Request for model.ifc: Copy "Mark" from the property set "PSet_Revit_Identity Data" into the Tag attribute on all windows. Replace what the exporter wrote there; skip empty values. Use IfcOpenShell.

First a look at what the model holds.

```python
import ifcopenshell
import ifcopenshell.util.element

model = ifcopenshell.open("model.ifc")
print(model.schema)
windows = model.by_type("IfcWindow")
print(len(windows), "windows")
for e in windows[:8]:
    source = ifcopenshell.util.element.get_pset(e, "PSet_Revit_Identity Data", "Mark")
    target = e.Tag
    print(e.id(), repr(source), repr(target), sep=" | ")
```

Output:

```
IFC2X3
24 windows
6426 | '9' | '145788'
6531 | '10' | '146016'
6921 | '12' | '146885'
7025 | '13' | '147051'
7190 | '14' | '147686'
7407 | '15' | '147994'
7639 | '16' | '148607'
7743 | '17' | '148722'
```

```python
import ifcopenshell
import ifcopenshell.util.element

model = ifcopenshell.open("model.ifc")

count = 0
for e in model.by_type("IfcWindow"):
    value = ifcopenshell.util.element.get_pset(e, "PSet_Revit_Identity Data", "Mark")
    current = e.Tag
    if not value or not value.strip() or current == value:
        continue
    e.Tag = value
    count += 1

print(count, "windows updated")

model.write("model_rev.ifc")
```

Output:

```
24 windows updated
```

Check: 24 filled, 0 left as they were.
